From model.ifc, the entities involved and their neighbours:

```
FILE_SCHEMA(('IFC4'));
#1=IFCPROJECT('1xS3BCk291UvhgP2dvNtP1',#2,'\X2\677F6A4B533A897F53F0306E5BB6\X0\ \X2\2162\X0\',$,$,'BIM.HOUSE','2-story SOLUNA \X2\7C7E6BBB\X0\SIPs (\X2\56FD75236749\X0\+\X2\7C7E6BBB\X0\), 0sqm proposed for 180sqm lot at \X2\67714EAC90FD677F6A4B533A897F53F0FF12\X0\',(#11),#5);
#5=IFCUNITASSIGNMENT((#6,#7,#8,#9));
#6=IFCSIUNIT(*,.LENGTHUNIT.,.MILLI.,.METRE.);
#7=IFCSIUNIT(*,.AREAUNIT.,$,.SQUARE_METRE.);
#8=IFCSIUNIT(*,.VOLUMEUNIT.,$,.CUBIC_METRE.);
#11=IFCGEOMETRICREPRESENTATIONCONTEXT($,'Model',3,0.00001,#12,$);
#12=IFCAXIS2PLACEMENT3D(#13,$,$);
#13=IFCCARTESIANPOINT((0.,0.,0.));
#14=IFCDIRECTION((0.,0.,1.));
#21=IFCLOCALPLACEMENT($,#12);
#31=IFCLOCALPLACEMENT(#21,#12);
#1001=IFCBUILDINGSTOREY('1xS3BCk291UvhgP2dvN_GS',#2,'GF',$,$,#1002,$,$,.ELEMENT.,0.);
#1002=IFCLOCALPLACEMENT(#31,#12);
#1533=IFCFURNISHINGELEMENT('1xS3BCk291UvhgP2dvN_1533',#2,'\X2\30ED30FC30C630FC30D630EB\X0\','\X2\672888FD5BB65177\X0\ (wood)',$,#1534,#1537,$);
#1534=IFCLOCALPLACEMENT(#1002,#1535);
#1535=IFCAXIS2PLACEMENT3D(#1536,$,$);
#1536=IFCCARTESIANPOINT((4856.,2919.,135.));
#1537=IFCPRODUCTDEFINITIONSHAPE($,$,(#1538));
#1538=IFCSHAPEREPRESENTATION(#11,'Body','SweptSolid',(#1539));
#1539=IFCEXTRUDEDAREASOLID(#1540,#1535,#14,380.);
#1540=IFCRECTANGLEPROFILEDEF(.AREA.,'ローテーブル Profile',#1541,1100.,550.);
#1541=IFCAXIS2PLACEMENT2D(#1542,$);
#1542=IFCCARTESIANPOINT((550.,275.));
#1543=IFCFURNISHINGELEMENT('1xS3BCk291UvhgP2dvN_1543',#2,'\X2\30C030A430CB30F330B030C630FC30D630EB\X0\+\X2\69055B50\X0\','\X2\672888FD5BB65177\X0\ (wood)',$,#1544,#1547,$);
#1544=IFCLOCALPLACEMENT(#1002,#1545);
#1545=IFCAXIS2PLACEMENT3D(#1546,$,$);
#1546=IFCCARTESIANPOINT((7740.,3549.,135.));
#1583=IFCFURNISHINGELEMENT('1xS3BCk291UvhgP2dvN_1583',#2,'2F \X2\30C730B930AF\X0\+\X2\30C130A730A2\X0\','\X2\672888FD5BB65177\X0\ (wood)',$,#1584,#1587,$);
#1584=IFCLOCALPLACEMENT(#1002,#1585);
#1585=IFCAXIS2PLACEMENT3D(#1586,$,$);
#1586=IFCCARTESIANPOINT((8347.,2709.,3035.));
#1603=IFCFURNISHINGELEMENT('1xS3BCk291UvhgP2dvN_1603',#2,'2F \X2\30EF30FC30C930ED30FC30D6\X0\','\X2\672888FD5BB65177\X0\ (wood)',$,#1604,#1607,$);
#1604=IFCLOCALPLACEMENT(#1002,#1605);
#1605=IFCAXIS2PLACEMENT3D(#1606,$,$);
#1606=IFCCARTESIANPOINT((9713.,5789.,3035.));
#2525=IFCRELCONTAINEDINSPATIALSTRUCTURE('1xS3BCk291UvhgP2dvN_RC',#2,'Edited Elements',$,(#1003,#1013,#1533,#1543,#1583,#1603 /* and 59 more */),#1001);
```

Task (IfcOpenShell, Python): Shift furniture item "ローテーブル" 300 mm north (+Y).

```python
import ifcopenshell
import ifcopenshell.api.geometry
import ifcopenshell.util.placement
import ifcopenshell.util.unit

model = ifcopenshell.open("model.ifc")
unit_scale = ifcopenshell.util.unit.calculate_unit_scale(model)

item = model.by_id(1533)
matrix = ifcopenshell.util.placement.get_local_placement(item.ObjectPlacement)
matrix[1, 3] += 0.3 / unit_scale
ifcopenshell.api.geometry.edit_object_placement(model, product=item, matrix=matrix, is_si=False)

print(ifcopenshell.util.placement.get_local_placement(item.ObjectPlacement).round(3) + 0.0)

model.write("model_edited.ifc")
```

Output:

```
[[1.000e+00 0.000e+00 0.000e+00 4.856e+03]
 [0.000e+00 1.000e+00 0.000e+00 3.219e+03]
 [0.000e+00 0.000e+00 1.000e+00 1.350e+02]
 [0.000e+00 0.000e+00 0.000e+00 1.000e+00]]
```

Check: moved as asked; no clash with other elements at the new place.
